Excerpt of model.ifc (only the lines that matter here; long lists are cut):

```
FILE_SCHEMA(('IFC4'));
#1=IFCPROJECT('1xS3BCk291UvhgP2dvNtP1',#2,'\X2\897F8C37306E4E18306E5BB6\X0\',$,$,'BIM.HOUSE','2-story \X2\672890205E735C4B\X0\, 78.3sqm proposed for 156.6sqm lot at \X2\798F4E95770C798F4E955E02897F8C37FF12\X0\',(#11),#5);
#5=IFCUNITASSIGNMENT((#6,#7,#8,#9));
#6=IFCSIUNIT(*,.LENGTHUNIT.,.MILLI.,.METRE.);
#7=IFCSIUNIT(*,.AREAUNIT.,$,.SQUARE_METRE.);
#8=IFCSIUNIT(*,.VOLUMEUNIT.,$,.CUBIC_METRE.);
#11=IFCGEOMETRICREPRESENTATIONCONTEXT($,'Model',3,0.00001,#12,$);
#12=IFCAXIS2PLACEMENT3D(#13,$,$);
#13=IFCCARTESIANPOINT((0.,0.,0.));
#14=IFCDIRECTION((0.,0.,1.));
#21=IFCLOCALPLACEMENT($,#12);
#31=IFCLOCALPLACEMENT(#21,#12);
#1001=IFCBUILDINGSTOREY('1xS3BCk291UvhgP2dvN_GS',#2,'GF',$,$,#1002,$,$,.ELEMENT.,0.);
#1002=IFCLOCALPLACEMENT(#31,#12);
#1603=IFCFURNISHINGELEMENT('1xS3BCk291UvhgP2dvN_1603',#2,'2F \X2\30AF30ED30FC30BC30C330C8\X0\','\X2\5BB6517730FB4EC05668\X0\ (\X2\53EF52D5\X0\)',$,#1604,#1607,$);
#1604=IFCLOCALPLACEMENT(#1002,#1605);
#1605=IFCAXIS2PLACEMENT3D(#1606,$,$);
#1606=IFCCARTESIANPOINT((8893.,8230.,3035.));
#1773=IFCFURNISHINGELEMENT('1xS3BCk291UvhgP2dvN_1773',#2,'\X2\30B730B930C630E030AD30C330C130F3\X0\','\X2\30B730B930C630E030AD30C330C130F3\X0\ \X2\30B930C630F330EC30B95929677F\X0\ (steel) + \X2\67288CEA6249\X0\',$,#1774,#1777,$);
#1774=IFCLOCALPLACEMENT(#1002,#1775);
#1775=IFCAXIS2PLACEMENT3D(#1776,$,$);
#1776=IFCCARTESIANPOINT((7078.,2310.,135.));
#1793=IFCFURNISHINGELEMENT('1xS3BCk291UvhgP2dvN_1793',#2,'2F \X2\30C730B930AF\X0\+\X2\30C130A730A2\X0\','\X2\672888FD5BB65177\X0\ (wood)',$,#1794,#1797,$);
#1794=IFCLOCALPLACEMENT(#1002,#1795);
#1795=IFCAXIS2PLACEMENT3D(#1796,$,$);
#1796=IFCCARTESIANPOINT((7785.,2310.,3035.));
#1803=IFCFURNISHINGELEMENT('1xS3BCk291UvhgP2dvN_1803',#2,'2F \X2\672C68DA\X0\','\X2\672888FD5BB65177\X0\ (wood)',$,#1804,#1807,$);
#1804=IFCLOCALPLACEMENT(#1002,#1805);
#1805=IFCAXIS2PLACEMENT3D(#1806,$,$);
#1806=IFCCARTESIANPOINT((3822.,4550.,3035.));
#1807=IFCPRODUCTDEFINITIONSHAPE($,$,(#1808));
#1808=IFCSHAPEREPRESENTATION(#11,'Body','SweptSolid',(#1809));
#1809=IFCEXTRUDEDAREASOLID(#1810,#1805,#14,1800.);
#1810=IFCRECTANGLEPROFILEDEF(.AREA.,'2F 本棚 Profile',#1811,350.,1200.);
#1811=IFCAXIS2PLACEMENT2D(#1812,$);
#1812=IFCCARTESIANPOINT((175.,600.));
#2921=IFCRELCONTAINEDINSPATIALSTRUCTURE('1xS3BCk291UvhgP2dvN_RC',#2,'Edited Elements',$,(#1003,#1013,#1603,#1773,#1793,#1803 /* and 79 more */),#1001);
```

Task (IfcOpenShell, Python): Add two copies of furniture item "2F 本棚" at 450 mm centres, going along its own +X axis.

```python
import ifcopenshell
import ifcopenshell.api.geometry
import ifcopenshell.api.root
import ifcopenshell.util.element
import ifcopenshell.util.placement

model = ifcopenshell.open("model.ifc")


def reuse_history(source, copy):
    """copy_class also copies each property set's owner history, people and application; keep the originals."""
    for rel in copy.IsDefinedBy:
        if rel.is_a("IfcRelDefinesByProperties") and (history := rel.RelatingPropertyDefinition.OwnerHistory):
            rel.RelatingPropertyDefinition.OwnerHistory = source.OwnerHistory
            ifcopenshell.util.element.remove_deep2(model, history)


source = model.by_guid("1xS3BCk291UvhgP2dvN_1803")
base = ifcopenshell.util.placement.get_local_placement(source.ObjectPlacement)
step = base[:3, 0] * 450.0

for i in range(1, 3):
    copy = ifcopenshell.api.root.copy_class(model, product=source)
    copy.Representation = ifcopenshell.util.element.copy_deep(
        model, source.Representation, exclude=["IfcGeometricRepresentationContext", "IfcRepresentationMap"]
    )
    reuse_history(source, copy)
    matrix = base.copy()
    matrix[:3, 3] += i * step
    print("added at", matrix[:3, 3].round(3) + 0.0)
    ifcopenshell.api.geometry.edit_object_placement(model, product=copy, matrix=matrix, is_si=False)

model.write("model_edited.ifc")
```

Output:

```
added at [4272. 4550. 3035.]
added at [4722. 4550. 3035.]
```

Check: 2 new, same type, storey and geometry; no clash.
